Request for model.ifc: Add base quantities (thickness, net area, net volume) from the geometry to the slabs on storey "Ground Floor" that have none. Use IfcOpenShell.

First a look at what the model holds.

```python
import ifcopenshell
import ifcopenshell.util.element
import ifcopenshell.util.unit

model = ifcopenshell.open("model.ifc")
print(model.schema)
for unit_type in ("LENGTHUNIT", "AREAUNIT", "VOLUMEUNIT"):
    print(unit_type, ifcopenshell.util.unit.calculate_unit_scale(model, unit_type))
storey = next(s for s in model.by_type("IfcBuildingStorey") if s.Name == "Ground Floor")
slabs = [e for e in ifcopenshell.util.element.get_decomposition(storey) if e.is_a("IfcSlab")]
for e in sorted(slabs, key=lambda e: e.id()):
    print(e.id(), e.is_a(), e.Name, list(ifcopenshell.util.element.get_psets(e, qtos_only=True)), sep=" | ")
```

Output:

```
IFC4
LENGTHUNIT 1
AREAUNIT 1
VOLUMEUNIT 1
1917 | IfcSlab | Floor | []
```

```python
import ifcopenshell
import ifcopenshell.api.pset
import ifcopenshell.geom
import ifcopenshell.util.element
import ifcopenshell.util.shape
import ifcopenshell.util.unit

model = ifcopenshell.open("model.ifc")
unit_scale = ifcopenshell.util.unit.calculate_unit_scale(model)
area_scale = ifcopenshell.util.unit.calculate_unit_scale(model, "AREAUNIT")
volume_scale = ifcopenshell.util.unit.calculate_unit_scale(model, "VOLUMEUNIT")
settings = ifcopenshell.geom.settings()

storey = next(s for s in model.by_type("IfcBuildingStorey") if s.Name == "Ground Floor")
slabs = [e for e in ifcopenshell.util.element.get_decomposition(storey) if e.is_a("IfcSlab")]

for e in sorted(slabs, key=lambda e: e.id()):
    if ifcopenshell.util.element.get_psets(e, qtos_only=True, should_inherit=False):
        continue
    # Geometry comes back in metres, in the element's own axes.
    shape = ifcopenshell.geom.create_shape(settings, e)
    values = {
        "Width": ifcopenshell.util.shape.get_z(shape.geometry) / unit_scale,
        "NetArea": ifcopenshell.util.shape.get_footprint_area(shape.geometry) / area_scale,
        "NetVolume": ifcopenshell.util.shape.get_volume(shape.geometry) / volume_scale,
    }
    qto = ifcopenshell.api.pset.add_qto(model, product=e, name="Qto_SlabBaseQuantities")
    ifcopenshell.api.pset.edit_qto(model, qto=qto, properties=values)
    print(e.id(), {k: round(v, 3) for k, v in values.items()})

model.write("model_updated.ifc")
```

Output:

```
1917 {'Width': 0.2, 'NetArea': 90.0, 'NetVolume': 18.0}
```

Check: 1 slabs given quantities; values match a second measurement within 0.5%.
